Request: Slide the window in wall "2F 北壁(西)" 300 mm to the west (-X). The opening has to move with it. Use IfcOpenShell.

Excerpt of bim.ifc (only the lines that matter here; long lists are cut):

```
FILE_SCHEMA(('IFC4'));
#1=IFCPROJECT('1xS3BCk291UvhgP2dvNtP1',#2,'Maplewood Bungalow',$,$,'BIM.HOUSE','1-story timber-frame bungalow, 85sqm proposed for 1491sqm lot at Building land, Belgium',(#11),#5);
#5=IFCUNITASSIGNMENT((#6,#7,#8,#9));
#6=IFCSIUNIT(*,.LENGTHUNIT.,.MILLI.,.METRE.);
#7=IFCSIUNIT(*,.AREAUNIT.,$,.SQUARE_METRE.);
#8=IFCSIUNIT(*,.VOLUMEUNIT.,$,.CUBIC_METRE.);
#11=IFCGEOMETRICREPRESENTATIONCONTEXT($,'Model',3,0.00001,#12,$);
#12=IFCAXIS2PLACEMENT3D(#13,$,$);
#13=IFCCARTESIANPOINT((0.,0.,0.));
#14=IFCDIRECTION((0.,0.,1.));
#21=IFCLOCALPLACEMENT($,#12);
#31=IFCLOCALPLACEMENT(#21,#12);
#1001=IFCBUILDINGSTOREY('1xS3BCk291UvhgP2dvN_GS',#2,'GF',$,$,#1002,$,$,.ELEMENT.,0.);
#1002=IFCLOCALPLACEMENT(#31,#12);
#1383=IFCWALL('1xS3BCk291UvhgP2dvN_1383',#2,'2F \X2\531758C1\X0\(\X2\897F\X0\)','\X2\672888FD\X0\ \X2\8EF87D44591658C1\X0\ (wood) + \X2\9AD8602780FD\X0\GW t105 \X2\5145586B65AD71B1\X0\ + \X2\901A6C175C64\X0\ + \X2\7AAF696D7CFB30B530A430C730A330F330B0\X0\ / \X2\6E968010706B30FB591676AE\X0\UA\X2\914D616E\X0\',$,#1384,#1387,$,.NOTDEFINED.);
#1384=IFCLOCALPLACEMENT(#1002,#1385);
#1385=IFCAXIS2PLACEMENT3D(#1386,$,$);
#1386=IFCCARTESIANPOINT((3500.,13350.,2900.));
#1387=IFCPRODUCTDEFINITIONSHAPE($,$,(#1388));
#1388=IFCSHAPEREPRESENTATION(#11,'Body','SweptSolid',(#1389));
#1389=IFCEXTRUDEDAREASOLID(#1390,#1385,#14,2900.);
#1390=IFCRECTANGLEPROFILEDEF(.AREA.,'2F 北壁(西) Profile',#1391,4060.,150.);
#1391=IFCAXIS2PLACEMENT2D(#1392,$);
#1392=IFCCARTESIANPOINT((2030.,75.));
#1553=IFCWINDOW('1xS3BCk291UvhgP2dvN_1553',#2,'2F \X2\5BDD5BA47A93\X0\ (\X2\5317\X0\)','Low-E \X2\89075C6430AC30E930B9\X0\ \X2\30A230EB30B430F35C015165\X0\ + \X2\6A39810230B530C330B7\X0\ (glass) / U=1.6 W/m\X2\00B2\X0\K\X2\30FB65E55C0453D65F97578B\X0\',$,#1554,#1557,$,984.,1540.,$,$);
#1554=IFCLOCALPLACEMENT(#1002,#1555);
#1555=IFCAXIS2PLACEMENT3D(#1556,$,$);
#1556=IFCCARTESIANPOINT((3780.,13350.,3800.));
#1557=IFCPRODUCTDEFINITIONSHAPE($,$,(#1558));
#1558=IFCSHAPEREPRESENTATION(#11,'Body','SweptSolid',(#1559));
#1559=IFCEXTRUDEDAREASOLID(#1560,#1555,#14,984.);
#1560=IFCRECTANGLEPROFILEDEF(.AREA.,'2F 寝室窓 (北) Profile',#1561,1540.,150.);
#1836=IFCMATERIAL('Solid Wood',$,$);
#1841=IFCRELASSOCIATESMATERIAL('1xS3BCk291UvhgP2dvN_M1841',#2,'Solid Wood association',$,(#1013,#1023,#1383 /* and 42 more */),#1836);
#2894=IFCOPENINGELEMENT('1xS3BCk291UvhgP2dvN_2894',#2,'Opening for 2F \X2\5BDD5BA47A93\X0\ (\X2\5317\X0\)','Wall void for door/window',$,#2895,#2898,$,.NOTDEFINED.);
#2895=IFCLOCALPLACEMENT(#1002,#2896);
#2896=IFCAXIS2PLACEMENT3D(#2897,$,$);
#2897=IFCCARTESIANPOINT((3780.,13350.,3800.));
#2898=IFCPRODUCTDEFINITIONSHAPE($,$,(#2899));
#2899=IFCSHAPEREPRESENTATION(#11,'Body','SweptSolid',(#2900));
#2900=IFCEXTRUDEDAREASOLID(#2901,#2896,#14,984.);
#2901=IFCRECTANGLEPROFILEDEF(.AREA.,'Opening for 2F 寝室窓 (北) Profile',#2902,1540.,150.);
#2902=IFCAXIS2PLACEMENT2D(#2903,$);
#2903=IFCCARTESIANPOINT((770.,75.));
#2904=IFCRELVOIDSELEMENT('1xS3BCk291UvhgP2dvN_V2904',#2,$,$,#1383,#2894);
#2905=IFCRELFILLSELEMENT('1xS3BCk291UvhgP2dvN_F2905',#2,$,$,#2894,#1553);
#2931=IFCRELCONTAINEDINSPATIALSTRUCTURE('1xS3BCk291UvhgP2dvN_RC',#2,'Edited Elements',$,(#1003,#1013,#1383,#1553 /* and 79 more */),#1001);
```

```python
import ifcopenshell
import ifcopenshell.api.geometry
import ifcopenshell.util.placement
import ifcopenshell.util.unit

model = ifcopenshell.open("bim.ifc")
unit_scale = ifcopenshell.util.unit.calculate_unit_scale(model)

window = model.by_id(1553)
opening = window.FillsVoids[0].RelatingOpeningElement
wall = opening.VoidsElements[0].RelatingBuildingElement

wall_matrix = ifcopenshell.util.placement.get_local_placement(wall.ObjectPlacement)
shift = wall_matrix[:3, 0] * -0.3 / unit_scale
before = ifcopenshell.util.placement.get_local_placement(window.ObjectPlacement)[:3, 3].copy()

# The window is not placed relative to its opening, so move both.
for product in (opening, window):
    matrix = ifcopenshell.util.placement.get_local_placement(product.ObjectPlacement)
    matrix[:3, 3] += shift
    ifcopenshell.api.geometry.edit_object_placement(model, product=product, matrix=matrix, is_si=False)

after = ifcopenshell.util.placement.get_local_placement(window.ObjectPlacement)[:3, 3]
print("window moved by", (after - before).round(3) + 0.0)

model.write("bim_edited.ifc")
```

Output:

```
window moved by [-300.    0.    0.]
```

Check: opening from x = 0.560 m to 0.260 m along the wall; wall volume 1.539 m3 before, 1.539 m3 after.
